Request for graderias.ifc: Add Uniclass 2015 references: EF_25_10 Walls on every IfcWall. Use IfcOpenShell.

First a look at what the model holds.

```python
import ifcopenshell

model = ifcopenshell.open("graderias.ifc")
print(model.schema)
print("classifications:", [c.Name for c in model.by_type("IfcClassification")])
for ifc_class in ("IfcDoor", "IfcRoof", "IfcStair", "IfcWall", "IfcWindow"):
    print(ifc_class, len(model.by_type(ifc_class)))
```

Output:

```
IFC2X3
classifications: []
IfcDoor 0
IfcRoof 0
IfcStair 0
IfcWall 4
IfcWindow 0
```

```python
import ifcopenshell
import ifcopenshell.api.classification

model = ifcopenshell.open("graderias.ifc")

# IFC2X3 requires Source and Edition and has no link from the project to the system.
system = model.create_entity("IfcClassification", Source="NBS", Edition="2015", Name="Uniclass 2015")

codes = {
    "IfcWall": ("EF_25_10", "Walls"),
}
for ifc_class, (code, name) in codes.items():
    products = model.by_type(ifc_class)
    ifcopenshell.api.classification.add_reference(
        model, products=products, classification=system, identification=code, name=name
    )
    print(code, len(products))

model.write("graderias_rev.ifc")
```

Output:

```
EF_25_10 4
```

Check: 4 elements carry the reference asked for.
